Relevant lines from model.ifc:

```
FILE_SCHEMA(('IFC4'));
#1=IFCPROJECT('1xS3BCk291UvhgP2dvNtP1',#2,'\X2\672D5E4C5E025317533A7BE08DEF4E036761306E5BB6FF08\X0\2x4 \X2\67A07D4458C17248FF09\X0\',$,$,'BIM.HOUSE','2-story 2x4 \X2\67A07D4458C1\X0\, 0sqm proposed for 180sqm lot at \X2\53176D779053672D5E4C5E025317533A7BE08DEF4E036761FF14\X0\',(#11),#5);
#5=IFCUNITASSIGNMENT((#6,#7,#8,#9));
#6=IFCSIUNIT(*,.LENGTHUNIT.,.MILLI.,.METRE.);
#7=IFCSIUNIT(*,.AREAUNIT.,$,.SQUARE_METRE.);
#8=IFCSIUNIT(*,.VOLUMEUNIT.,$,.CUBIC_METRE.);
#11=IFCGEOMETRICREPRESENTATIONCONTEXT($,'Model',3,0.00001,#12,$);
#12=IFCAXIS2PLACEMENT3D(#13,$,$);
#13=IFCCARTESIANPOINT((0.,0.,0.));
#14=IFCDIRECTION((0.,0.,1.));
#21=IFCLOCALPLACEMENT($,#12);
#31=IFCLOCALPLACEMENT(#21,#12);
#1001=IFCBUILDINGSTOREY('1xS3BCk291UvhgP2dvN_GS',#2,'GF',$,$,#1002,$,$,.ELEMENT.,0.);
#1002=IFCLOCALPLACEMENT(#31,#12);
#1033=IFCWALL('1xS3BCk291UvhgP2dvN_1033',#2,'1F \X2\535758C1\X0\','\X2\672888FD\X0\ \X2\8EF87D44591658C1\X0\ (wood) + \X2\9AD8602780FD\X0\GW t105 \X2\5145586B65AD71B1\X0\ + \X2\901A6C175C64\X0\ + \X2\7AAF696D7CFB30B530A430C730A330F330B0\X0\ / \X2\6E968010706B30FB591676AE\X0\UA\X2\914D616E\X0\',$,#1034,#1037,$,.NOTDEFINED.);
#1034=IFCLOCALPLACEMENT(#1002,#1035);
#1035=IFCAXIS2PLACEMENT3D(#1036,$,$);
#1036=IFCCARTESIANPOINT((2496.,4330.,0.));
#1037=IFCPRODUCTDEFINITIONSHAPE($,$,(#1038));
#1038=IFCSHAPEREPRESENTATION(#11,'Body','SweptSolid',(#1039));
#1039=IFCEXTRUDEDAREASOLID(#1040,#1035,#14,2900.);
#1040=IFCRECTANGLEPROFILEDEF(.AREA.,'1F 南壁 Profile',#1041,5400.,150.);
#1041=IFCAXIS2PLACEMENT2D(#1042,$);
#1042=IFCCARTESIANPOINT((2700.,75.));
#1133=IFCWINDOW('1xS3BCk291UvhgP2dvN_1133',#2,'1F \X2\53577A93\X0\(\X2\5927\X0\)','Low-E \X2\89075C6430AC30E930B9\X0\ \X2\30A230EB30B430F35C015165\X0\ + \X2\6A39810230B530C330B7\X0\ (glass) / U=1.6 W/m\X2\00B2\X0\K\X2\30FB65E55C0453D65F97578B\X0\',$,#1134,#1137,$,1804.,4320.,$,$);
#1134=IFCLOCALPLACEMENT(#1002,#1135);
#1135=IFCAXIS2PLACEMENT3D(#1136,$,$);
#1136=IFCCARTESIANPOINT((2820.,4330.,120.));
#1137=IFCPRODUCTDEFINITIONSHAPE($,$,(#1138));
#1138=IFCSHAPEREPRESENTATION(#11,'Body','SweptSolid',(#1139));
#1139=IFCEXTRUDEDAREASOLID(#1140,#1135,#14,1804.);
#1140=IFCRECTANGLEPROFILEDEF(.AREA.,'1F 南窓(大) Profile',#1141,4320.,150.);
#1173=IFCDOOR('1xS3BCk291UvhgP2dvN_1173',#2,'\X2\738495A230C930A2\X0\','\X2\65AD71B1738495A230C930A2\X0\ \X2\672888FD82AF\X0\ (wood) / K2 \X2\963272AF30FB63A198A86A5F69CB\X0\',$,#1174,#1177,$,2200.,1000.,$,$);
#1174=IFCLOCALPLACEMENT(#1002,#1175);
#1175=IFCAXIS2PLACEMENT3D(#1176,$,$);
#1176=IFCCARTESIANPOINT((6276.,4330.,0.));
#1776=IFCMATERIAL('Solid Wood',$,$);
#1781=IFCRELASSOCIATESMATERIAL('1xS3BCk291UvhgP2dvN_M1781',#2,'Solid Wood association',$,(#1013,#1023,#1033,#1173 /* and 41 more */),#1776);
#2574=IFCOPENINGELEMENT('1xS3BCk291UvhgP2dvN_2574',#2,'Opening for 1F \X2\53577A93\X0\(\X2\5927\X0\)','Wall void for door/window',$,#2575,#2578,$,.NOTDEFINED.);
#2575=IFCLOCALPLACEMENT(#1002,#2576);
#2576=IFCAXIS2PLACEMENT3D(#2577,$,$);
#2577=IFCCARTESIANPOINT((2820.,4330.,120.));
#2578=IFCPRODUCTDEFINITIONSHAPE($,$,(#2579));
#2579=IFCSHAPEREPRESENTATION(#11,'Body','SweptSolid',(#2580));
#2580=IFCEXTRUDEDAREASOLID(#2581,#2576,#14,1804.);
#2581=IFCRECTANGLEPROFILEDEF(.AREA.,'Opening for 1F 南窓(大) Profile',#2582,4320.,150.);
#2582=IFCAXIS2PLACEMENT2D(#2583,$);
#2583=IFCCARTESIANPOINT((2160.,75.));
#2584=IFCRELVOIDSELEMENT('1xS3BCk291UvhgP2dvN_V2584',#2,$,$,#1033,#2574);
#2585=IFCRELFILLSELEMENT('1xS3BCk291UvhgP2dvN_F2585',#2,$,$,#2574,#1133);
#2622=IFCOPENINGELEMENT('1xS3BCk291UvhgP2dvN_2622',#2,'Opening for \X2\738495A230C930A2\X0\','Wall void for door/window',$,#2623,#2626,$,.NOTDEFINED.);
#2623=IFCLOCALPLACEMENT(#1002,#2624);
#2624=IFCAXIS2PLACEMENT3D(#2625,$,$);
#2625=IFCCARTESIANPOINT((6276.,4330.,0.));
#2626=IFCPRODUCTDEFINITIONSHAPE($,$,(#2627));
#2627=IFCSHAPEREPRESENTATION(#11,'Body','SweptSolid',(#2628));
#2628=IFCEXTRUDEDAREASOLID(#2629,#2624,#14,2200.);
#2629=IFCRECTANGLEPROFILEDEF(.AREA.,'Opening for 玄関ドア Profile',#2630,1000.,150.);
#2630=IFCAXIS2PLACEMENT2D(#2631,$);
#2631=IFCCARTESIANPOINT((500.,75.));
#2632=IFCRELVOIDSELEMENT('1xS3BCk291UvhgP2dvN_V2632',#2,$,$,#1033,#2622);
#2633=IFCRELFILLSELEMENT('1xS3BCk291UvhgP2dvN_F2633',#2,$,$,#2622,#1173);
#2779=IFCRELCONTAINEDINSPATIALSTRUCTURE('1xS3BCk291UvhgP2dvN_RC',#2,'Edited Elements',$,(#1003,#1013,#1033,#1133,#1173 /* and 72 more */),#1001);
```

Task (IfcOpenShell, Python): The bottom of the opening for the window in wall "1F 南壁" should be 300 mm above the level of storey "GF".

```python
import numpy as np
import ifcopenshell
import ifcopenshell.api.geometry
import ifcopenshell.geom
import ifcopenshell.util.element
import ifcopenshell.util.placement
import ifcopenshell.util.shape
import ifcopenshell.util.unit

model = ifcopenshell.open("model.ifc")
unit_scale = ifcopenshell.util.unit.calculate_unit_scale(model)

window = model.by_id(1133)
opening = window.FillsVoids[0].RelatingOpeningElement
storey = ifcopenshell.util.element.get_container(window, ifc_class="IfcBuildingStorey")
level = ifcopenshell.util.placement.get_local_placement(storey.ObjectPlacement)[2, 3]

# The opening's origin need not be at the sill, so measure its lowest point.
shape = ifcopenshell.geom.create_shape(ifcopenshell.geom.settings(), opening)
bottom = ifcopenshell.util.shape.get_shape_bottom_elevation(shape, shape.geometry) / unit_scale
dz = level + 0.3 / unit_scale - bottom

shift = np.array([0.0, 0.0, dz])
# The window is not placed relative to its opening, so move both.
for product in (opening, window):
    matrix = ifcopenshell.util.placement.get_local_placement(product.ObjectPlacement)
    matrix[:3, 3] += shift
    ifcopenshell.api.geometry.edit_object_placement(model, product=product, matrix=matrix, is_si=False)

print(f"moved by {dz * unit_scale:+.3f} m")

model.write("model-out.ifc")
```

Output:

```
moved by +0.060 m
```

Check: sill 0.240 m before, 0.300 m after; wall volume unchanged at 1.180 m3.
